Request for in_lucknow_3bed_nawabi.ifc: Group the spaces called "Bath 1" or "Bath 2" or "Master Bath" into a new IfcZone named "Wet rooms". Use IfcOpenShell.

First a look at what the model holds.

```python
import ifcopenshell

model = ifcopenshell.open("in_lucknow_3bed_nawabi.ifc")
print(model.schema)
seen = {}
for space in model.by_type("IfcSpace"):
    seen[space.LongName] = seen.get(space.LongName, 0) + 1
for name, count in sorted(seen.items(), key=str):
    print(count, "x", name)
print("zones:", [z.Name for z in model.by_type("IfcZone")][:20])
```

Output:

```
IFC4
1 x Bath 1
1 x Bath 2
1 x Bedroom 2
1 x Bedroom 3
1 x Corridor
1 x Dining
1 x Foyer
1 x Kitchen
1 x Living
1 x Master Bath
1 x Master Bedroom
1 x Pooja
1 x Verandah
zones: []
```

```python
import ifcopenshell
import ifcopenshell.api.group
import ifcopenshell.api.root

model = ifcopenshell.open("in_lucknow_3bed_nawabi.ifc")

names = {"Bath 1", "Bath 2", "Master Bath"}
spaces = [s for s in model.by_type("IfcSpace") if s.LongName in names]

zone = ifcopenshell.api.root.create_entity(model, ifc_class="IfcZone", name="Wet rooms")
ifcopenshell.api.group.assign_group(model, products=spaces, group=zone)
print(len(spaces), "spaces in", zone.Name)

model.write("in_lucknow_3bed_nawabi_updated.ifc")
```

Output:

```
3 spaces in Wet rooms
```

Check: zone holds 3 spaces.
